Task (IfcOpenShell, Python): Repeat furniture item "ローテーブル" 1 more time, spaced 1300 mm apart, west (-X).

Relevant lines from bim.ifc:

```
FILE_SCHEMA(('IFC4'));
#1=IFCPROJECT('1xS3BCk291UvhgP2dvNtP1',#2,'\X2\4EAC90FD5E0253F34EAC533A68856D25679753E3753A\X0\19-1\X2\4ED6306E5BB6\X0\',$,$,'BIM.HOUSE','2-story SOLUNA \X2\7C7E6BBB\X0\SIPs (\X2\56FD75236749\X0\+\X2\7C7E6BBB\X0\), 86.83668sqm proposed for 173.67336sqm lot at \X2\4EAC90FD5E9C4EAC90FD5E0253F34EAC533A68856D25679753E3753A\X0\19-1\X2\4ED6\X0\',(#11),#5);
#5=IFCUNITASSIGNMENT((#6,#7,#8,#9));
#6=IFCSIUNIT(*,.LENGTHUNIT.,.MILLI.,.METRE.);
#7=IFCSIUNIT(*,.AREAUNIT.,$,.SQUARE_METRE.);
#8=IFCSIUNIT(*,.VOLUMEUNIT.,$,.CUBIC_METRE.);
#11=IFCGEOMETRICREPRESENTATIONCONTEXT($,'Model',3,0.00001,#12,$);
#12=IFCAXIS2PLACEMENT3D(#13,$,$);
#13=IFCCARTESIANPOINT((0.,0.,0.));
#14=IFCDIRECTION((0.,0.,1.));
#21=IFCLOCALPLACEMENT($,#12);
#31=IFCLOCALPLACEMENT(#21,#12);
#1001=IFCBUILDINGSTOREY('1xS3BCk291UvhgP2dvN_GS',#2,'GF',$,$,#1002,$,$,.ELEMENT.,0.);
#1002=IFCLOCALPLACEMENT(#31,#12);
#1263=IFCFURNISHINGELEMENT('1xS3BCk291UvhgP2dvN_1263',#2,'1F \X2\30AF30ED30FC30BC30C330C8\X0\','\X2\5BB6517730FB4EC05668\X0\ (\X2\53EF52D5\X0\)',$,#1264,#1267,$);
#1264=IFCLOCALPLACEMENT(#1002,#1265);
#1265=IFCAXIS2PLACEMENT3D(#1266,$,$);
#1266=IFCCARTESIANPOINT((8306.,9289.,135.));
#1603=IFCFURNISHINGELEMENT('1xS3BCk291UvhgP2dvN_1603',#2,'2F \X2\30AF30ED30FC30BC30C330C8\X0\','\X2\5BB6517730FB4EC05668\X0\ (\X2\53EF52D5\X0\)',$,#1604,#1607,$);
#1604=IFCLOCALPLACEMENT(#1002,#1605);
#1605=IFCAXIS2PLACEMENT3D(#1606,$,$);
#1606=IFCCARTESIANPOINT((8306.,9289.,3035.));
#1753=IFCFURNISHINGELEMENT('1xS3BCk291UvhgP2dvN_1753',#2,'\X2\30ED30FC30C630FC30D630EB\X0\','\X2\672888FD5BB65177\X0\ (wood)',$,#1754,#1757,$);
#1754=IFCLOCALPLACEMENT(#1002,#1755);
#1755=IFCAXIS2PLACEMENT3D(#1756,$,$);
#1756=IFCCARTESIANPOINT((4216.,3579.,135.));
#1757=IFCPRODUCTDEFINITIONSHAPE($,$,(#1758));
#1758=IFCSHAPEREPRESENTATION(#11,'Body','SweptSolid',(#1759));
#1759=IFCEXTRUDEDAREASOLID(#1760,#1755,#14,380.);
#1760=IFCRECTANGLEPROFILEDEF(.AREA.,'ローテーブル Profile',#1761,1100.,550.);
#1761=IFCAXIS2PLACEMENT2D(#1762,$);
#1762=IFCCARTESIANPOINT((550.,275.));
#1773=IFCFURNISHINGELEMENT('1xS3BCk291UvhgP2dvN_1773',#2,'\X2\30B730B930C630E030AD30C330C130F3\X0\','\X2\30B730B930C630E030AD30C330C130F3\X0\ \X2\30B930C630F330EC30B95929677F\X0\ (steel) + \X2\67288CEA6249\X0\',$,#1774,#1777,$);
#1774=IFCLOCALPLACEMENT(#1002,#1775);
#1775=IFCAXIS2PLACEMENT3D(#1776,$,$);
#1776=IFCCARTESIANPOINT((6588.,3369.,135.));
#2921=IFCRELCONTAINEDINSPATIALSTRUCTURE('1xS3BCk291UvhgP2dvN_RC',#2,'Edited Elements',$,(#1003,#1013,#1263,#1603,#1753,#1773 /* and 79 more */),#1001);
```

```python
import numpy as np
import ifcopenshell
import ifcopenshell.api.geometry
import ifcopenshell.api.root
import ifcopenshell.util.element
import ifcopenshell.util.placement
import ifcopenshell.util.unit

model = ifcopenshell.open("bim.ifc")
unit_scale = ifcopenshell.util.unit.calculate_unit_scale(model)


def reuse_history(source, copy):
    """copy_class also copies each property set's owner history, people and application; keep the originals."""
    for rel in copy.IsDefinedBy:
        if rel.is_a("IfcRelDefinesByProperties") and (history := rel.RelatingPropertyDefinition.OwnerHistory):
            rel.RelatingPropertyDefinition.OwnerHistory = source.OwnerHistory
            ifcopenshell.util.element.remove_deep2(model, history)


source = model.by_guid("1xS3BCk291UvhgP2dvN_1753")
base = ifcopenshell.util.placement.get_local_placement(source.ObjectPlacement)
step = np.array([-1.0, 0.0, 0.0]) * 1.3 / unit_scale

for i in range(1, 2):
    copy = ifcopenshell.api.root.copy_class(model, product=source)
    copy.Representation = ifcopenshell.util.element.copy_deep(
        model, source.Representation, exclude=["IfcGeometricRepresentationContext", "IfcRepresentationMap"]
    )
    reuse_history(source, copy)
    matrix = base.copy()
    matrix[:3, 3] += i * step
    print("added at", matrix[:3, 3].round(3) + 0.0)
    ifcopenshell.api.geometry.edit_object_placement(model, product=copy, matrix=matrix, is_si=False)

model.write("bim-out.ifc")
```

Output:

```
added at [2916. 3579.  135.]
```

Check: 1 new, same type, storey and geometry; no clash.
